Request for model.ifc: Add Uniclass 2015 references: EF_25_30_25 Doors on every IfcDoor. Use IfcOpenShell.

First a look at what the model holds.

```python
import ifcopenshell

model = ifcopenshell.open("model.ifc")
print(model.schema)
print("classifications:", [c.Name for c in model.by_type("IfcClassification")])
for ifc_class in ("IfcDoor", "IfcRoof", "IfcStair", "IfcWall", "IfcWindow"):
    print(ifc_class, len(model.by_type(ifc_class)))
```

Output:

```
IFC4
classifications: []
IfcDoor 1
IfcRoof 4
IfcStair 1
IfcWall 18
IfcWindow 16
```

```python
import ifcopenshell
import ifcopenshell.api.classification

model = ifcopenshell.open("model.ifc")

system = ifcopenshell.api.classification.add_classification(model, classification="Uniclass 2015")

codes = {
    "IfcDoor": ("EF_25_30_25", "Doors"),
}
for ifc_class, (code, name) in codes.items():
    products = model.by_type(ifc_class)
    ifcopenshell.api.classification.add_reference(
        model, products=products, classification=system, identification=code, name=name
    )
    print(code, len(products))

model.write("model-out.ifc")
```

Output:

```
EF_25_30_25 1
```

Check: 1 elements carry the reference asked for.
